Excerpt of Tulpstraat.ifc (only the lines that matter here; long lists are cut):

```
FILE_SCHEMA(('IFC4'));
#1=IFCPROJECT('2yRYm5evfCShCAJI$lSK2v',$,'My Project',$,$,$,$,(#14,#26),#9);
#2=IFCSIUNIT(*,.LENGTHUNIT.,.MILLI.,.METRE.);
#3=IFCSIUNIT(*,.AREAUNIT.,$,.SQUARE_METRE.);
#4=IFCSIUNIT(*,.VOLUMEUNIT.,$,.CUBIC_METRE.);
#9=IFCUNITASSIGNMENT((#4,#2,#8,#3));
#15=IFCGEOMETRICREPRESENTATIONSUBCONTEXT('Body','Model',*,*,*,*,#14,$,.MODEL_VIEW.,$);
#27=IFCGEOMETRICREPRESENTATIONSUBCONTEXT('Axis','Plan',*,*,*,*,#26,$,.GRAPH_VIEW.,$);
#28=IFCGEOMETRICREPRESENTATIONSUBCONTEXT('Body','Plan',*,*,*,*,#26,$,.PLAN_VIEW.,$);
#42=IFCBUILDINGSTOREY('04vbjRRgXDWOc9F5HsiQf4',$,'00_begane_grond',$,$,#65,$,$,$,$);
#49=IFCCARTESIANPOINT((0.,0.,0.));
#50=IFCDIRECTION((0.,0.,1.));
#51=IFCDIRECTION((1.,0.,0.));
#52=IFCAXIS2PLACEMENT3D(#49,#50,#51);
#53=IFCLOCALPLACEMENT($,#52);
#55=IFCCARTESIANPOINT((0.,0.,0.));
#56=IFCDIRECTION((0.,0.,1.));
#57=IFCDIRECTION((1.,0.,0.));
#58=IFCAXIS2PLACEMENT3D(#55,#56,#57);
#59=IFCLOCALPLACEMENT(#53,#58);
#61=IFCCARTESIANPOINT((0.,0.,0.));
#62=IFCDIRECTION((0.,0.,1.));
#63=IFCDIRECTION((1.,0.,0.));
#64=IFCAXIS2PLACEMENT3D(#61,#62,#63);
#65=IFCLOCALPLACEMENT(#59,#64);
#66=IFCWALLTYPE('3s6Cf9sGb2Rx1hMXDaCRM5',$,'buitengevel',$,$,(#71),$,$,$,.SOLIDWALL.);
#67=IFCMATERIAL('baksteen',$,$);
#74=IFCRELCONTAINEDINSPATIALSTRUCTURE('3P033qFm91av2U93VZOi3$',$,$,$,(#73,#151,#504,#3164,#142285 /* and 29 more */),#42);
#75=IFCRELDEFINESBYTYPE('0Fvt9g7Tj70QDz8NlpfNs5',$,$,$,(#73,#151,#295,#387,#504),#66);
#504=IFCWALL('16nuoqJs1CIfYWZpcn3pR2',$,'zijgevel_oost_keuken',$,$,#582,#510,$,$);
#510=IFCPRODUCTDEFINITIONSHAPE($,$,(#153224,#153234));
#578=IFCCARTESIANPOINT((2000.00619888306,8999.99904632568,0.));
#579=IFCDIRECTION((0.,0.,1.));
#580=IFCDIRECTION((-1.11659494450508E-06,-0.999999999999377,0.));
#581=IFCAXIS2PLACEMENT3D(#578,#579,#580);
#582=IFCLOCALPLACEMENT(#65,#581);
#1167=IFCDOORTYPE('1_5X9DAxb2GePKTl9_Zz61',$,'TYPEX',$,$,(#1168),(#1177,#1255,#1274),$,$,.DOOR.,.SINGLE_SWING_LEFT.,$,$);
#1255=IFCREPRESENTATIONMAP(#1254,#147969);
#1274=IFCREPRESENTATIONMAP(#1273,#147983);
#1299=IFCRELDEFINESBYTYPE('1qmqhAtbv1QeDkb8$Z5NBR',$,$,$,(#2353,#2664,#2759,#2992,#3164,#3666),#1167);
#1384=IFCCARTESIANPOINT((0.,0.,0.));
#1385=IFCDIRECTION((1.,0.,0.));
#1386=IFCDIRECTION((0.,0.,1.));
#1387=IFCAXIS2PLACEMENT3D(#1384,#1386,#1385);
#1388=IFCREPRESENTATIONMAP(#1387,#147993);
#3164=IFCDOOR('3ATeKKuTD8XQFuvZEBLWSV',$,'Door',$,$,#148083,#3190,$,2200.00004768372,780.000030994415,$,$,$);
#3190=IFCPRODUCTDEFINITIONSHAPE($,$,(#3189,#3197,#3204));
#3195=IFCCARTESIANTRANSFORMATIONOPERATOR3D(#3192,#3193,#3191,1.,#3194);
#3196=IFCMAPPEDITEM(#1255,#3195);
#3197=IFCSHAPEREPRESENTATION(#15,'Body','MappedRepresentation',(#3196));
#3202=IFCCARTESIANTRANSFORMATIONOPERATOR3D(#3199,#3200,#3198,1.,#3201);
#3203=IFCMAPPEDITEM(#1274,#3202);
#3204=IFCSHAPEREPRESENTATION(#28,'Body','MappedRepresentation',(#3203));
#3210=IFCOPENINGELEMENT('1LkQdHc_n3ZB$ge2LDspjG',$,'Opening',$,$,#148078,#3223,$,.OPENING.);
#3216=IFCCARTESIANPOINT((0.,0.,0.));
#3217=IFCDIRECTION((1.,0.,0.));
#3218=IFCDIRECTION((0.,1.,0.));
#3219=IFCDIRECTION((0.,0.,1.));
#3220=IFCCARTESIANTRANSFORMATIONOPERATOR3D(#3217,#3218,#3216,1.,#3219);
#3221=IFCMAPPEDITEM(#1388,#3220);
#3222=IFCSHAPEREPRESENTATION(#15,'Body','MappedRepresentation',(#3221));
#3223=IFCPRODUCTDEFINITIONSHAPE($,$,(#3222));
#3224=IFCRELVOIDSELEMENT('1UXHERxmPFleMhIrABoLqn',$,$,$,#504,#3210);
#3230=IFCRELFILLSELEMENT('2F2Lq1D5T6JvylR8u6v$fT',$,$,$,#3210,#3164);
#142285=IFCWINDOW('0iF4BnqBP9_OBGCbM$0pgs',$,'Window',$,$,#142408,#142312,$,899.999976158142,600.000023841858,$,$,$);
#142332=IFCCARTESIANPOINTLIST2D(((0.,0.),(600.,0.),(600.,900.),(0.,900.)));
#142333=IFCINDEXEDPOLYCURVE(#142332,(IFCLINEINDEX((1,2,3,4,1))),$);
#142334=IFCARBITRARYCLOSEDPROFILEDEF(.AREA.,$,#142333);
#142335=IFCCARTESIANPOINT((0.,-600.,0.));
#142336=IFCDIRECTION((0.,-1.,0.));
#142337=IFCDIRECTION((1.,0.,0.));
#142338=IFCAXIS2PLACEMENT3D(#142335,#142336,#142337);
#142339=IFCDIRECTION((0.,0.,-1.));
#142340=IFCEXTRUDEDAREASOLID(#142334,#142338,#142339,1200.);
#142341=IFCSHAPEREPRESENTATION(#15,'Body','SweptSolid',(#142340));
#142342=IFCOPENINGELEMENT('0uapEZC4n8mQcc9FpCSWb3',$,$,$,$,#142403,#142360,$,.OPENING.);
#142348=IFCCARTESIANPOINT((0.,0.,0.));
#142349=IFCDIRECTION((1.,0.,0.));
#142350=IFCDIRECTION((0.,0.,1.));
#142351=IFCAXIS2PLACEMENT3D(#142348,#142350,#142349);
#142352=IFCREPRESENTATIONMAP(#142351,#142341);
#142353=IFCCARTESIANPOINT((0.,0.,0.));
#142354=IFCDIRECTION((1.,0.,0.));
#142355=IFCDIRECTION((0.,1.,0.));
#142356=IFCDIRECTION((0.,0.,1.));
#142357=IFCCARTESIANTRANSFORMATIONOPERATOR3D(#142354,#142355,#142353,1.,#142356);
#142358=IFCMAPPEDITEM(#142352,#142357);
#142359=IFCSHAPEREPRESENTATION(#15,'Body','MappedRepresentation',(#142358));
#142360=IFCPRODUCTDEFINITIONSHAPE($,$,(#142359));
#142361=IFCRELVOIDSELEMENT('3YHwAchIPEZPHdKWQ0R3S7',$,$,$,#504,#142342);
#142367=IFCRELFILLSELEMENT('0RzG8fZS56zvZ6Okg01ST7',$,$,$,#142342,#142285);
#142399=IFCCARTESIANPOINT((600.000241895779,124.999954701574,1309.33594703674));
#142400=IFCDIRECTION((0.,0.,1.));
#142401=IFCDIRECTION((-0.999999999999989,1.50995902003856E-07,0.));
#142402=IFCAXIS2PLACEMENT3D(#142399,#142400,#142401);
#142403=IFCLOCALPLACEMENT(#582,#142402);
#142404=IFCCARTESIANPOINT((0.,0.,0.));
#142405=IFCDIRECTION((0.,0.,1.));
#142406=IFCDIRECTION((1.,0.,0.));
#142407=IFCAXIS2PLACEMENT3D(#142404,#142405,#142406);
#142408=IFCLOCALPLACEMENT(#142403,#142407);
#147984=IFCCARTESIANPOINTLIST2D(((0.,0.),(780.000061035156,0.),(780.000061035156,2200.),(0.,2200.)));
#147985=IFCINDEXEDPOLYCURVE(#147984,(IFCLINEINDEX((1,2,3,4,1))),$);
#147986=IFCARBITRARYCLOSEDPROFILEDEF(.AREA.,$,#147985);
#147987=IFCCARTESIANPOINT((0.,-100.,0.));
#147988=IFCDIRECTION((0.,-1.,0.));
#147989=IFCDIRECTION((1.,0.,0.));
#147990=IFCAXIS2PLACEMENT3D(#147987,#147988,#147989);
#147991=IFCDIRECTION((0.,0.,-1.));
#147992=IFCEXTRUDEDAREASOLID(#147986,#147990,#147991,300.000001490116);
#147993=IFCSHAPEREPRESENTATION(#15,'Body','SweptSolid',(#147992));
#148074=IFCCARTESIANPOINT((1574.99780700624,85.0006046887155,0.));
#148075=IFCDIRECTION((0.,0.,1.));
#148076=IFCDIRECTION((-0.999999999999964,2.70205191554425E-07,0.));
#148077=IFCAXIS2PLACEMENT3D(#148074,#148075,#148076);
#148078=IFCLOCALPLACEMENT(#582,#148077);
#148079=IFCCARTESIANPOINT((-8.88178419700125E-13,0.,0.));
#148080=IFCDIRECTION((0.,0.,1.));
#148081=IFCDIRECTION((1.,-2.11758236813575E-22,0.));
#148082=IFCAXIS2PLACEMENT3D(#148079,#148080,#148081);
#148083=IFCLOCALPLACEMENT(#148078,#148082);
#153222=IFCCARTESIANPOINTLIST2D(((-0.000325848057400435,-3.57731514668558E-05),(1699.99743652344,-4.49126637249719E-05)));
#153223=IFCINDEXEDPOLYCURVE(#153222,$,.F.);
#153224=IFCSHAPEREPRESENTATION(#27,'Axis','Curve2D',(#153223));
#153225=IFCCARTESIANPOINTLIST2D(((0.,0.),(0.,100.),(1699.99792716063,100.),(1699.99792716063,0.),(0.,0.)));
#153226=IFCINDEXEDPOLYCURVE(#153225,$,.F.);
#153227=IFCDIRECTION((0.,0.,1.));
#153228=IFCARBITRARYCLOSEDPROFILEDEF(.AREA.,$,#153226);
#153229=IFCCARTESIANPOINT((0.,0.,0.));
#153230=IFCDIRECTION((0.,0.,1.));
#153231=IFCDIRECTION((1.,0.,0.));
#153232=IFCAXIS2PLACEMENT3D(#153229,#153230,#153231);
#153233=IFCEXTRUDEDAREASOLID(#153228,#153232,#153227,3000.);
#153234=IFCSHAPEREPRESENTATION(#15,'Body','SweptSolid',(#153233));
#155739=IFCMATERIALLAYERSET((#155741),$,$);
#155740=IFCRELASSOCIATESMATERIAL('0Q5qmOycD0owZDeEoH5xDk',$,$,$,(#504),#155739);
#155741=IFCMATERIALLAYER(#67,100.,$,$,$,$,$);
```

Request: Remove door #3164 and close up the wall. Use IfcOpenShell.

```python
import ifcopenshell
import ifcopenshell.api.feature
import ifcopenshell.api.root
import ifcopenshell.geom
import ifcopenshell.util.shape

model = ifcopenshell.open("Tulpstraat.ifc")
settings = ifcopenshell.geom.settings()


def volume(element):
    """Net volume in cubic metres, openings subtracted."""
    shape = ifcopenshell.geom.create_shape(settings, element)
    return ifcopenshell.util.shape.get_volume(shape.geometry)


door = model.by_guid("3ATeKKuTD8XQFuvZEBLWSV")
opening = door.FillsVoids[0].RelatingOpeningElement
wall = opening.VoidsElements[0].RelatingBuildingElement
before = volume(wall)

ifcopenshell.api.root.remove_product(model, product=door)
ifcopenshell.api.feature.remove_feature(model, feature=opening)

after = volume(wall)

print(f"wall volume {before:.3f} -> {after:.3f} m3")

model.write("Tulpstraat_edited.ifc")
```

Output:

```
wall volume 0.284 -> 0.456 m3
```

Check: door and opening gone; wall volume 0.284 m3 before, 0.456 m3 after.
